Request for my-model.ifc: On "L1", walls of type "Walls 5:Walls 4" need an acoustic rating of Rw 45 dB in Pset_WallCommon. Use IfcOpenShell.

First a look at what the model holds.

```python
import ifcopenshell
import ifcopenshell.util.element

model = ifcopenshell.open("my-model.ifc")
print(model.schema)
storey = next(s for s in model.by_type("IfcBuildingStorey") if s.Name == "L1")
walls = [e for e in ifcopenshell.util.element.get_decomposition(storey) if e.is_a("IfcWall")]
seen = {}
for e in walls:
    element_type = ifcopenshell.util.element.get_type(e)
    key = (element_type.Name if element_type != e and element_type else None, ifcopenshell.util.element.get_pset(e, "Pset_WallCommon", "AcousticRating"))
    seen[key] = seen.get(key, 0) + 1
for (name, value), count in sorted(seen.items(), key=str):
    print(count, "x", name, "|", value)
```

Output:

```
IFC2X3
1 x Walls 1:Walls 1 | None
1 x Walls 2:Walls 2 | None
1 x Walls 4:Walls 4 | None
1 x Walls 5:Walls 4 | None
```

```python
import ifcopenshell
import ifcopenshell.api.pset
import ifcopenshell.util.element

model = ifcopenshell.open("my-model.ifc")

storey = next(s for s in model.by_type("IfcBuildingStorey") if s.Name == "L1")
walls = [e for e in ifcopenshell.util.element.get_decomposition(storey) if e.is_a("IfcWall")]

count = 0
for e in walls:
    element_type = ifcopenshell.util.element.get_type(e)
    if element_type in (None, e) or element_type.Name != "Walls 5:Walls 4":
        continue
    # add_pset returns the element's existing set when there is one.
    pset = ifcopenshell.api.pset.add_pset(model, product=e, name="Pset_WallCommon")
    ifcopenshell.api.pset.edit_pset(model, pset=pset, properties={"AcousticRating": "Rw 45 dB"})
    count += 1

print(count, "walls updated")

model.write("my-model_edited.ifc")
```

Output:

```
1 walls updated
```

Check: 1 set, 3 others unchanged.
